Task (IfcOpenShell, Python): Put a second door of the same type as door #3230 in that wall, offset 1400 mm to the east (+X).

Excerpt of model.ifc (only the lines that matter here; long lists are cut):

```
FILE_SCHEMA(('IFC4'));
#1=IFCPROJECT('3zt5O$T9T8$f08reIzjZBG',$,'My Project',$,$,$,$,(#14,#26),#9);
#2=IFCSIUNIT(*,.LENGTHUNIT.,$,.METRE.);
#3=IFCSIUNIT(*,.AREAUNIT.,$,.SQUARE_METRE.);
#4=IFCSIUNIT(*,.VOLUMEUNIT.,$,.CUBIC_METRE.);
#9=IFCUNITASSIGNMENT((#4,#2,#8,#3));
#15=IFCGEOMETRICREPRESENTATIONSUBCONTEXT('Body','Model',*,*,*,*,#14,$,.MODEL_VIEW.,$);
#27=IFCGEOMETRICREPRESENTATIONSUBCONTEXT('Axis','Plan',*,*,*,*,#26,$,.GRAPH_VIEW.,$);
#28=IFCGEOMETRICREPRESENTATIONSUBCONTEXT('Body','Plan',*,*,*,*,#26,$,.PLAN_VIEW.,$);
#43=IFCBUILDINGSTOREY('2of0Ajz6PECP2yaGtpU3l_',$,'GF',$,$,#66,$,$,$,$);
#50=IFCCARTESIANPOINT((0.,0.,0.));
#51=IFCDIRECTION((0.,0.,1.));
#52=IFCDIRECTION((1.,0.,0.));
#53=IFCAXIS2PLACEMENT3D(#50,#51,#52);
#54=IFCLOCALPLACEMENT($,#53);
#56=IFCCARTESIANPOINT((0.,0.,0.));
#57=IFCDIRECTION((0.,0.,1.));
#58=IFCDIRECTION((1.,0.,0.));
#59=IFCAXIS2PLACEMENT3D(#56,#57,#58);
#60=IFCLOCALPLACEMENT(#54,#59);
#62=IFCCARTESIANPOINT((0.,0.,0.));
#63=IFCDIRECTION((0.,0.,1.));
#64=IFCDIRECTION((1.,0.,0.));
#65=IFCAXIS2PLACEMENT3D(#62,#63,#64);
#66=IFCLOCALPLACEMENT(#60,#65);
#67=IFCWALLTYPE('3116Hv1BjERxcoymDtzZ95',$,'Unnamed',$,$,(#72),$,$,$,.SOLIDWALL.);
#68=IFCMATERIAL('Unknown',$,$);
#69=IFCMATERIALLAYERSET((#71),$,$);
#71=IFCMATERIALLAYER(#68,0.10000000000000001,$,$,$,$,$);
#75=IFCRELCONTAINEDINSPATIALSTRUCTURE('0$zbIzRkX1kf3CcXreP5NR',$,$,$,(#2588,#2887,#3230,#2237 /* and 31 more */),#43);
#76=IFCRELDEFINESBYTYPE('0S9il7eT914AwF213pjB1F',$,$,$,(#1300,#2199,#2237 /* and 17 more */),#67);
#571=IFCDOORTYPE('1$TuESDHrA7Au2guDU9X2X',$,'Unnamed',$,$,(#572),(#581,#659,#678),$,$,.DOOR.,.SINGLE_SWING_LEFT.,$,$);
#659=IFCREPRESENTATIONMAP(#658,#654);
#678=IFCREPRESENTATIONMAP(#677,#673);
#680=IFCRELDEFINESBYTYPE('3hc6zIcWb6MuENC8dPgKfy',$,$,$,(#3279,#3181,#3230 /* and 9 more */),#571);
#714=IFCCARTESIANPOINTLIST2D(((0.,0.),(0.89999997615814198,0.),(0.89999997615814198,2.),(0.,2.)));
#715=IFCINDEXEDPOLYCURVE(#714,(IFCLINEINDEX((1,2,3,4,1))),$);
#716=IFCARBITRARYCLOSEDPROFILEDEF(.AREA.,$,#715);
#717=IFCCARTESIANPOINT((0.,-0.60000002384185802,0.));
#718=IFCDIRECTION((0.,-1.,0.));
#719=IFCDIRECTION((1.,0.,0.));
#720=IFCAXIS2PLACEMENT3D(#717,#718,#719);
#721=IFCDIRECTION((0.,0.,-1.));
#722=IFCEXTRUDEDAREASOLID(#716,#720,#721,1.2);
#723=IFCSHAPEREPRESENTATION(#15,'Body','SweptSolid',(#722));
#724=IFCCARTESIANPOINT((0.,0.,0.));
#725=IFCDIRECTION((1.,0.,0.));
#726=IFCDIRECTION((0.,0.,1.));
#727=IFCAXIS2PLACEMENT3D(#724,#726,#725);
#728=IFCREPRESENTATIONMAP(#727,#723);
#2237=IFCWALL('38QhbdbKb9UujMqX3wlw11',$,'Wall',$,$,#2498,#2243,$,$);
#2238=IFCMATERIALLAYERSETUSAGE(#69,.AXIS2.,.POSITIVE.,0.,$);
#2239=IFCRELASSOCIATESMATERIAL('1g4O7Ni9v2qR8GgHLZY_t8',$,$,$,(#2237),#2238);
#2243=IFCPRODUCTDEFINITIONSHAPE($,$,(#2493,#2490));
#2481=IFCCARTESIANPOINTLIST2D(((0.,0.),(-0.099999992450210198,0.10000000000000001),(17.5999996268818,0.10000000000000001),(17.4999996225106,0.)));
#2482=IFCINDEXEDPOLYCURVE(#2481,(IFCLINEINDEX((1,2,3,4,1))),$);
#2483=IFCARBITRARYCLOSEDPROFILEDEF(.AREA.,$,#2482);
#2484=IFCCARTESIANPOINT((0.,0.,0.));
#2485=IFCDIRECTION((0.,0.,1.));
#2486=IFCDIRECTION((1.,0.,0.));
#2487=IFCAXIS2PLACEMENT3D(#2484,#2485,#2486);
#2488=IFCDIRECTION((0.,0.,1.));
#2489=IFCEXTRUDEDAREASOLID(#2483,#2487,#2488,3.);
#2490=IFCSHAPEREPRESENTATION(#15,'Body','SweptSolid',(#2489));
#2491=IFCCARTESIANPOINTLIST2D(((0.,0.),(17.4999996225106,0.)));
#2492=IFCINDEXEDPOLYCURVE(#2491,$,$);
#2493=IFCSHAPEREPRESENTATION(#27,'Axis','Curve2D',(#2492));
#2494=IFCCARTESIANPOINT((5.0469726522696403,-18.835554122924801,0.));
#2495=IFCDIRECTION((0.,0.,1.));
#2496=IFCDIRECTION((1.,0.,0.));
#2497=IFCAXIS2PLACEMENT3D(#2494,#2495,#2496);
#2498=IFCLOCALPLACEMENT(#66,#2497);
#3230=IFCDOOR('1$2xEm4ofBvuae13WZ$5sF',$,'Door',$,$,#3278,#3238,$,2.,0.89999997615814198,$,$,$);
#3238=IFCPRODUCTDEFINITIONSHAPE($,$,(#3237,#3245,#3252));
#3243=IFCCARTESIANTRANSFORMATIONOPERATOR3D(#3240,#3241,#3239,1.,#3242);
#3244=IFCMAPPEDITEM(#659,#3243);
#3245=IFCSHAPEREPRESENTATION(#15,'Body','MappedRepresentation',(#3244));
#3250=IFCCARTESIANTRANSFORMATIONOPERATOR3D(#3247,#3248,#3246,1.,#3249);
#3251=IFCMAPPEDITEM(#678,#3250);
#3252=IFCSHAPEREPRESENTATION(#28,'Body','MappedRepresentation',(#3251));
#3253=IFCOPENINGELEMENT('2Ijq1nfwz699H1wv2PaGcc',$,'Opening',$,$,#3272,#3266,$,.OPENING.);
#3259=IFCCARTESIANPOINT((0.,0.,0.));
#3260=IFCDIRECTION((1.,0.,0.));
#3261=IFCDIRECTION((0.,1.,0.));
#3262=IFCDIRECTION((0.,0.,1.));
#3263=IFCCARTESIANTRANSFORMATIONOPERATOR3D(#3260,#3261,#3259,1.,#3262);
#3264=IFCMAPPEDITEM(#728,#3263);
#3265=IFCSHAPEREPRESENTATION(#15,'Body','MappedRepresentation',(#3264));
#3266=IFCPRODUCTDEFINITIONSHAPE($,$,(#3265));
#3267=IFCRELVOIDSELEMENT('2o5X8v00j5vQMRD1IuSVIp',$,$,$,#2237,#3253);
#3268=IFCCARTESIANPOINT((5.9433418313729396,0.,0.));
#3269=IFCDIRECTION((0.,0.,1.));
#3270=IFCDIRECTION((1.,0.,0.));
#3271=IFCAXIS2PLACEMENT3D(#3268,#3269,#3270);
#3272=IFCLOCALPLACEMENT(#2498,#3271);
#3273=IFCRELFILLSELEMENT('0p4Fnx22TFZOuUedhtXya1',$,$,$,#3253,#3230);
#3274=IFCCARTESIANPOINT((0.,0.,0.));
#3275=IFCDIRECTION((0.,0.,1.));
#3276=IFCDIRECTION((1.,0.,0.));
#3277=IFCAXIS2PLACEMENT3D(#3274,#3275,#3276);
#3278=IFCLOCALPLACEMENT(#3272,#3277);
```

```python
import ifcopenshell
import ifcopenshell.api.feature
import ifcopenshell.api.geometry
import ifcopenshell.api.root
import ifcopenshell.geom
import ifcopenshell.util.element
import ifcopenshell.util.placement
import ifcopenshell.util.shape

model = ifcopenshell.open("model.ifc")
settings = ifcopenshell.geom.settings()


def volume(element):
    """Net volume in cubic metres, openings subtracted."""
    shape = ifcopenshell.geom.create_shape(settings, element)
    return ifcopenshell.util.shape.get_volume(shape.geometry)


door = model.by_guid("1$2xEm4ofBvuae13WZ$5sF")
opening = door.FillsVoids[0].RelatingOpeningElement
wall = opening.VoidsElements[0].RelatingBuildingElement
before = volume(wall)
shift = ifcopenshell.util.placement.get_local_placement(wall.ObjectPlacement)[:3, 0] * 1.4

# copy_class copies the void relationship, type, container and properties, but no geometry.
new_opening = ifcopenshell.api.root.copy_class(model, product=opening)
new_opening.Representation = ifcopenshell.util.element.copy_deep(
    model, opening.Representation, exclude=["IfcGeometricRepresentationContext", "IfcRepresentationMap"]
)
new_door = ifcopenshell.api.root.copy_class(model, product=door)
new_door.Representation = ifcopenshell.util.element.copy_deep(
    model, door.Representation, exclude=["IfcGeometricRepresentationContext", "IfcRepresentationMap"]
)
ifcopenshell.api.feature.add_filling(model, opening=new_opening, element=new_door)

for old, new in ((opening, new_opening), (door, new_door)):
    matrix = ifcopenshell.util.placement.get_local_placement(old.ObjectPlacement)
    matrix[:3, 3] += shift
    ifcopenshell.api.geometry.edit_object_placement(model, product=new, matrix=matrix, is_si=False)

after = volume(wall)

print(f"wall volume {before:.3f} -> {after:.3f} m3")

model.write("model-out.ifc")
```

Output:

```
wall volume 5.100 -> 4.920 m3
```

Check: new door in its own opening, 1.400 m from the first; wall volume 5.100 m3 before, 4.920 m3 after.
